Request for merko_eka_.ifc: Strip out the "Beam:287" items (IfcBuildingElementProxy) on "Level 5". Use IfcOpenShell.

First a look at what the model holds.

```python
import ifcopenshell
import ifcopenshell.util.element

model = ifcopenshell.open("merko_eka_.ifc")
print(model.schema)
storey = next(s for s in model.by_type("IfcBuildingStorey") if s.Name == "Level 5")
proxies = [e for e in ifcopenshell.util.element.get_decomposition(storey) if e.is_a("IfcBuildingElementProxy")]
seen = {}
for e in proxies:
    element_type = ifcopenshell.util.element.get_type(e)
    name = element_type.Name if element_type not in (None, e) else None
    seen[name] = seen.get(name, 0) + 1
for name, count in sorted(seen.items(), key=str):
    print(count, "x", name)
```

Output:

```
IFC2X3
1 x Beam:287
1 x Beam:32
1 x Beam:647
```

```python
import ifcopenshell
import ifcopenshell.api.root
import ifcopenshell.util.element

model = ifcopenshell.open("merko_eka_.ifc")

storey = next(s for s in model.by_type("IfcBuildingStorey") if s.Name == "Level 5")
proxies = [e for e in ifcopenshell.util.element.get_decomposition(storey) if e.is_a("IfcBuildingElementProxy")]
targets = [e for e in proxies if (t := ifcopenshell.util.element.get_type(e)) not in (None, e) and t.Name == "Beam:287"]

for e in targets:
    ifcopenshell.api.root.remove_product(model, product=e)
print(len(targets), "removed")

model.write("merko_eka__updated.ifc")
```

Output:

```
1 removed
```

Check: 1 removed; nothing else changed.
